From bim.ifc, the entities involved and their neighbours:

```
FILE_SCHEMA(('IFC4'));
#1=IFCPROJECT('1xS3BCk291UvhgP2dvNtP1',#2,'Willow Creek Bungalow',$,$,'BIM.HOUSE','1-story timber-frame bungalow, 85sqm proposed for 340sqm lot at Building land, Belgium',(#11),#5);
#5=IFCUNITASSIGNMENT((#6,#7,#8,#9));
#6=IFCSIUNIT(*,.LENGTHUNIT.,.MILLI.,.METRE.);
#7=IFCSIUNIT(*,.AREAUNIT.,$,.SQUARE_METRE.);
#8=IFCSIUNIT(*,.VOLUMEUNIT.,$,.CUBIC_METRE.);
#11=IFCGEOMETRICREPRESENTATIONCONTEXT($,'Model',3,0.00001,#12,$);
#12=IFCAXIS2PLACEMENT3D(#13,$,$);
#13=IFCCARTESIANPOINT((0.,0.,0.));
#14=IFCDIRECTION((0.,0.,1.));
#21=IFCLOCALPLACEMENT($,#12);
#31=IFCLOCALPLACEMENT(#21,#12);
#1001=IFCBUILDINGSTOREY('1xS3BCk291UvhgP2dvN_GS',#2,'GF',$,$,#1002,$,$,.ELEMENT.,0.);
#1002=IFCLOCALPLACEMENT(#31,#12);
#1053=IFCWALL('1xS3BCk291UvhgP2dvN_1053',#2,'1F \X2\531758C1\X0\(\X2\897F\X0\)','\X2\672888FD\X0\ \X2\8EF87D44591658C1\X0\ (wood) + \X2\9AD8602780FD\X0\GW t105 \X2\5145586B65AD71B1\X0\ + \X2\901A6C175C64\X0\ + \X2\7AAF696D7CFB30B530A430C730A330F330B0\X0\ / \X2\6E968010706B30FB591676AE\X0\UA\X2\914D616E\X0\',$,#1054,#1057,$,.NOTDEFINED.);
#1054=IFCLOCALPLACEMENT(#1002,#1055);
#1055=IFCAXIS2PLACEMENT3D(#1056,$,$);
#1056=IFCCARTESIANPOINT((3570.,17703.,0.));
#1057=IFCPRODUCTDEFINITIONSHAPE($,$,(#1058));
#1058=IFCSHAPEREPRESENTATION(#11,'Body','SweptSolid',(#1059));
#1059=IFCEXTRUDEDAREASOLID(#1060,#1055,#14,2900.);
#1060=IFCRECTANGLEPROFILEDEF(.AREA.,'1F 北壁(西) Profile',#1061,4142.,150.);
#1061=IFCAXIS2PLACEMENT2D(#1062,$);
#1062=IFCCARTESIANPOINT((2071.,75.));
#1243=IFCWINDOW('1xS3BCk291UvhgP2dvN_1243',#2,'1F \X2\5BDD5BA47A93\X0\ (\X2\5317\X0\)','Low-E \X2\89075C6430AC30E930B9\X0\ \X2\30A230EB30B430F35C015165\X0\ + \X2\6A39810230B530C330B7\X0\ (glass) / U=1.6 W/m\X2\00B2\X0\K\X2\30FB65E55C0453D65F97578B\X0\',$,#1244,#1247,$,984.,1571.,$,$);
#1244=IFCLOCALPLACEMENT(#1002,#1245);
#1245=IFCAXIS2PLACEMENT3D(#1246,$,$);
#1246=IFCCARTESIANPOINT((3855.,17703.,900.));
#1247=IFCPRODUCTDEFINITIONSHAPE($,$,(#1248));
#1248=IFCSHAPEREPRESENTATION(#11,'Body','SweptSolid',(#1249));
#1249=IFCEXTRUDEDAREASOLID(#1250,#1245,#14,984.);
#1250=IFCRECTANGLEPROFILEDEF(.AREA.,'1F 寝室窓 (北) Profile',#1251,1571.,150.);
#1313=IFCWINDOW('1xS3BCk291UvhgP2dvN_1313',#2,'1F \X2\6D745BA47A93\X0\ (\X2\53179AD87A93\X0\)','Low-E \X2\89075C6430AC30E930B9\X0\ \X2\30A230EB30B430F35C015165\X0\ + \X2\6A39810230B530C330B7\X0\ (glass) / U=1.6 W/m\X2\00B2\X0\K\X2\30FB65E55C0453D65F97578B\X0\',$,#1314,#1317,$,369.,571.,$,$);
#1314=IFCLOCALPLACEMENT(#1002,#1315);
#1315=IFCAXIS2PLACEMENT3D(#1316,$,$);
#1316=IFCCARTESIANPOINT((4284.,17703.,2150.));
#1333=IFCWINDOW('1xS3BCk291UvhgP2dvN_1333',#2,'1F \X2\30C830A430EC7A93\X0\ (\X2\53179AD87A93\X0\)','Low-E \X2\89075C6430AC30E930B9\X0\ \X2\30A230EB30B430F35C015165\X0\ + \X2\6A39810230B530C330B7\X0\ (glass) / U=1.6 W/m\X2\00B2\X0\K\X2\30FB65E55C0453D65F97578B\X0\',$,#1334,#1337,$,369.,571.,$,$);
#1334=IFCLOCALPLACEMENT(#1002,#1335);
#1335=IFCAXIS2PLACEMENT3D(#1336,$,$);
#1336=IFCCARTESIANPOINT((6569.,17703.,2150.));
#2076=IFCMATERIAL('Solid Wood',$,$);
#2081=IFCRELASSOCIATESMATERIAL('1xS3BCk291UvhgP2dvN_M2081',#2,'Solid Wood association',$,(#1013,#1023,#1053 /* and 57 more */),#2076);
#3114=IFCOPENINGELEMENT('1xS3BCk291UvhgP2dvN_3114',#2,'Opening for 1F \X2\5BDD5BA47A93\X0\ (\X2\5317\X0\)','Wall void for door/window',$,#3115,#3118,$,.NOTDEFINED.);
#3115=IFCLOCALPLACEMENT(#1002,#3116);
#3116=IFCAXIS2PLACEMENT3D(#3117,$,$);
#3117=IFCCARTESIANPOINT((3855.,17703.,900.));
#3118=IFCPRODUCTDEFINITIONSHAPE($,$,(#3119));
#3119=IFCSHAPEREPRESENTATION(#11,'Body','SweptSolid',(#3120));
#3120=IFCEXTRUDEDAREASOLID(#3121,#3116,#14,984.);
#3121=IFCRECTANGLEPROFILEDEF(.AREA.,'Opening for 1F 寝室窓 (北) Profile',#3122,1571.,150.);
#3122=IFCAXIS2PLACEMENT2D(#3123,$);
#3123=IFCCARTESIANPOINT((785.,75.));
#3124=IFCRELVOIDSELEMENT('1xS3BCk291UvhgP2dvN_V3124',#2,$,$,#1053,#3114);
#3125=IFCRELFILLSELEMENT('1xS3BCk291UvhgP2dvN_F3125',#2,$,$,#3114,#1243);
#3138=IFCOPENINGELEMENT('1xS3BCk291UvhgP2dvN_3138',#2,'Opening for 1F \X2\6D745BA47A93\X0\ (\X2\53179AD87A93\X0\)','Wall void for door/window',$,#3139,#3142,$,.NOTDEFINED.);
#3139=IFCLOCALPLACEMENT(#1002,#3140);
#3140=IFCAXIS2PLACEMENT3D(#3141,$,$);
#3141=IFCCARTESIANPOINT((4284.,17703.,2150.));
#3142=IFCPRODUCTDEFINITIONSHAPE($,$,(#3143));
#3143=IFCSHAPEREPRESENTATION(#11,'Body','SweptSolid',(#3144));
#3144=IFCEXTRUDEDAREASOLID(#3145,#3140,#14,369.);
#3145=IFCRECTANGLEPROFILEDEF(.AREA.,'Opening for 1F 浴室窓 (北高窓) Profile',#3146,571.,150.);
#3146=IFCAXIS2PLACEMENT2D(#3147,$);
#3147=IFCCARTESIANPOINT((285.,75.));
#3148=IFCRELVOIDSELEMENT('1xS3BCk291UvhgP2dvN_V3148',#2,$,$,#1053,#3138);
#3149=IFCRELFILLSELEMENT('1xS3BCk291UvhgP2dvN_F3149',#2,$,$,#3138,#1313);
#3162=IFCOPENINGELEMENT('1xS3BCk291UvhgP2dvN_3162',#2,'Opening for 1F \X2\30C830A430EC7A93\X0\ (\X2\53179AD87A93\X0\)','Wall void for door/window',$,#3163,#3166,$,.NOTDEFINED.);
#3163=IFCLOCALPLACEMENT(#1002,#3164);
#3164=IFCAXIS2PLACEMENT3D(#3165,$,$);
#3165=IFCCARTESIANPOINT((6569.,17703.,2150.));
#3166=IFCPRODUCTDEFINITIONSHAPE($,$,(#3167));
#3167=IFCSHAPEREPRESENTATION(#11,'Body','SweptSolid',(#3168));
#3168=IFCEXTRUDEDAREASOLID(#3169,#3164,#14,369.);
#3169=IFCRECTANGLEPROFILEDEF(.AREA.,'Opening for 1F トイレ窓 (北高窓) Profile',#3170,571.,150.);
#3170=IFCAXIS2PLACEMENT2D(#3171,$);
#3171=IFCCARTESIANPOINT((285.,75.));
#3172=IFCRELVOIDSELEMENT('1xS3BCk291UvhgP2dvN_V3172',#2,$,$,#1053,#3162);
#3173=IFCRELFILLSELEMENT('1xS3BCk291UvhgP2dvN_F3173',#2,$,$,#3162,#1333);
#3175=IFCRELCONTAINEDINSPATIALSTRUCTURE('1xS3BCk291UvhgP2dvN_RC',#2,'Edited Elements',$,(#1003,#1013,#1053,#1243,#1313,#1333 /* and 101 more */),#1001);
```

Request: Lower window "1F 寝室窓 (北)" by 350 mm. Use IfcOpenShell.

```python
import numpy as np
import ifcopenshell
import ifcopenshell.api.geometry
import ifcopenshell.util.placement
import ifcopenshell.util.unit

model = ifcopenshell.open("bim.ifc")
unit_scale = ifcopenshell.util.unit.calculate_unit_scale(model)

window = model.by_guid("1xS3BCk291UvhgP2dvN_1243")
opening = window.FillsVoids[0].RelatingOpeningElement
dz = -0.35 / unit_scale

shift = np.array([0.0, 0.0, dz])
# The window is not placed relative to its opening, so move both.
for product in (opening, window):
    matrix = ifcopenshell.util.placement.get_local_placement(product.ObjectPlacement)
    matrix[:3, 3] += shift
    ifcopenshell.api.geometry.edit_object_placement(model, product=product, matrix=matrix, is_si=False)

print(f"moved by {dz * unit_scale:+.3f} m")

model.write("bim_rev.ifc")
```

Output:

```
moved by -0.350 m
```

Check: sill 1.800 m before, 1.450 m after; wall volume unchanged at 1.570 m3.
